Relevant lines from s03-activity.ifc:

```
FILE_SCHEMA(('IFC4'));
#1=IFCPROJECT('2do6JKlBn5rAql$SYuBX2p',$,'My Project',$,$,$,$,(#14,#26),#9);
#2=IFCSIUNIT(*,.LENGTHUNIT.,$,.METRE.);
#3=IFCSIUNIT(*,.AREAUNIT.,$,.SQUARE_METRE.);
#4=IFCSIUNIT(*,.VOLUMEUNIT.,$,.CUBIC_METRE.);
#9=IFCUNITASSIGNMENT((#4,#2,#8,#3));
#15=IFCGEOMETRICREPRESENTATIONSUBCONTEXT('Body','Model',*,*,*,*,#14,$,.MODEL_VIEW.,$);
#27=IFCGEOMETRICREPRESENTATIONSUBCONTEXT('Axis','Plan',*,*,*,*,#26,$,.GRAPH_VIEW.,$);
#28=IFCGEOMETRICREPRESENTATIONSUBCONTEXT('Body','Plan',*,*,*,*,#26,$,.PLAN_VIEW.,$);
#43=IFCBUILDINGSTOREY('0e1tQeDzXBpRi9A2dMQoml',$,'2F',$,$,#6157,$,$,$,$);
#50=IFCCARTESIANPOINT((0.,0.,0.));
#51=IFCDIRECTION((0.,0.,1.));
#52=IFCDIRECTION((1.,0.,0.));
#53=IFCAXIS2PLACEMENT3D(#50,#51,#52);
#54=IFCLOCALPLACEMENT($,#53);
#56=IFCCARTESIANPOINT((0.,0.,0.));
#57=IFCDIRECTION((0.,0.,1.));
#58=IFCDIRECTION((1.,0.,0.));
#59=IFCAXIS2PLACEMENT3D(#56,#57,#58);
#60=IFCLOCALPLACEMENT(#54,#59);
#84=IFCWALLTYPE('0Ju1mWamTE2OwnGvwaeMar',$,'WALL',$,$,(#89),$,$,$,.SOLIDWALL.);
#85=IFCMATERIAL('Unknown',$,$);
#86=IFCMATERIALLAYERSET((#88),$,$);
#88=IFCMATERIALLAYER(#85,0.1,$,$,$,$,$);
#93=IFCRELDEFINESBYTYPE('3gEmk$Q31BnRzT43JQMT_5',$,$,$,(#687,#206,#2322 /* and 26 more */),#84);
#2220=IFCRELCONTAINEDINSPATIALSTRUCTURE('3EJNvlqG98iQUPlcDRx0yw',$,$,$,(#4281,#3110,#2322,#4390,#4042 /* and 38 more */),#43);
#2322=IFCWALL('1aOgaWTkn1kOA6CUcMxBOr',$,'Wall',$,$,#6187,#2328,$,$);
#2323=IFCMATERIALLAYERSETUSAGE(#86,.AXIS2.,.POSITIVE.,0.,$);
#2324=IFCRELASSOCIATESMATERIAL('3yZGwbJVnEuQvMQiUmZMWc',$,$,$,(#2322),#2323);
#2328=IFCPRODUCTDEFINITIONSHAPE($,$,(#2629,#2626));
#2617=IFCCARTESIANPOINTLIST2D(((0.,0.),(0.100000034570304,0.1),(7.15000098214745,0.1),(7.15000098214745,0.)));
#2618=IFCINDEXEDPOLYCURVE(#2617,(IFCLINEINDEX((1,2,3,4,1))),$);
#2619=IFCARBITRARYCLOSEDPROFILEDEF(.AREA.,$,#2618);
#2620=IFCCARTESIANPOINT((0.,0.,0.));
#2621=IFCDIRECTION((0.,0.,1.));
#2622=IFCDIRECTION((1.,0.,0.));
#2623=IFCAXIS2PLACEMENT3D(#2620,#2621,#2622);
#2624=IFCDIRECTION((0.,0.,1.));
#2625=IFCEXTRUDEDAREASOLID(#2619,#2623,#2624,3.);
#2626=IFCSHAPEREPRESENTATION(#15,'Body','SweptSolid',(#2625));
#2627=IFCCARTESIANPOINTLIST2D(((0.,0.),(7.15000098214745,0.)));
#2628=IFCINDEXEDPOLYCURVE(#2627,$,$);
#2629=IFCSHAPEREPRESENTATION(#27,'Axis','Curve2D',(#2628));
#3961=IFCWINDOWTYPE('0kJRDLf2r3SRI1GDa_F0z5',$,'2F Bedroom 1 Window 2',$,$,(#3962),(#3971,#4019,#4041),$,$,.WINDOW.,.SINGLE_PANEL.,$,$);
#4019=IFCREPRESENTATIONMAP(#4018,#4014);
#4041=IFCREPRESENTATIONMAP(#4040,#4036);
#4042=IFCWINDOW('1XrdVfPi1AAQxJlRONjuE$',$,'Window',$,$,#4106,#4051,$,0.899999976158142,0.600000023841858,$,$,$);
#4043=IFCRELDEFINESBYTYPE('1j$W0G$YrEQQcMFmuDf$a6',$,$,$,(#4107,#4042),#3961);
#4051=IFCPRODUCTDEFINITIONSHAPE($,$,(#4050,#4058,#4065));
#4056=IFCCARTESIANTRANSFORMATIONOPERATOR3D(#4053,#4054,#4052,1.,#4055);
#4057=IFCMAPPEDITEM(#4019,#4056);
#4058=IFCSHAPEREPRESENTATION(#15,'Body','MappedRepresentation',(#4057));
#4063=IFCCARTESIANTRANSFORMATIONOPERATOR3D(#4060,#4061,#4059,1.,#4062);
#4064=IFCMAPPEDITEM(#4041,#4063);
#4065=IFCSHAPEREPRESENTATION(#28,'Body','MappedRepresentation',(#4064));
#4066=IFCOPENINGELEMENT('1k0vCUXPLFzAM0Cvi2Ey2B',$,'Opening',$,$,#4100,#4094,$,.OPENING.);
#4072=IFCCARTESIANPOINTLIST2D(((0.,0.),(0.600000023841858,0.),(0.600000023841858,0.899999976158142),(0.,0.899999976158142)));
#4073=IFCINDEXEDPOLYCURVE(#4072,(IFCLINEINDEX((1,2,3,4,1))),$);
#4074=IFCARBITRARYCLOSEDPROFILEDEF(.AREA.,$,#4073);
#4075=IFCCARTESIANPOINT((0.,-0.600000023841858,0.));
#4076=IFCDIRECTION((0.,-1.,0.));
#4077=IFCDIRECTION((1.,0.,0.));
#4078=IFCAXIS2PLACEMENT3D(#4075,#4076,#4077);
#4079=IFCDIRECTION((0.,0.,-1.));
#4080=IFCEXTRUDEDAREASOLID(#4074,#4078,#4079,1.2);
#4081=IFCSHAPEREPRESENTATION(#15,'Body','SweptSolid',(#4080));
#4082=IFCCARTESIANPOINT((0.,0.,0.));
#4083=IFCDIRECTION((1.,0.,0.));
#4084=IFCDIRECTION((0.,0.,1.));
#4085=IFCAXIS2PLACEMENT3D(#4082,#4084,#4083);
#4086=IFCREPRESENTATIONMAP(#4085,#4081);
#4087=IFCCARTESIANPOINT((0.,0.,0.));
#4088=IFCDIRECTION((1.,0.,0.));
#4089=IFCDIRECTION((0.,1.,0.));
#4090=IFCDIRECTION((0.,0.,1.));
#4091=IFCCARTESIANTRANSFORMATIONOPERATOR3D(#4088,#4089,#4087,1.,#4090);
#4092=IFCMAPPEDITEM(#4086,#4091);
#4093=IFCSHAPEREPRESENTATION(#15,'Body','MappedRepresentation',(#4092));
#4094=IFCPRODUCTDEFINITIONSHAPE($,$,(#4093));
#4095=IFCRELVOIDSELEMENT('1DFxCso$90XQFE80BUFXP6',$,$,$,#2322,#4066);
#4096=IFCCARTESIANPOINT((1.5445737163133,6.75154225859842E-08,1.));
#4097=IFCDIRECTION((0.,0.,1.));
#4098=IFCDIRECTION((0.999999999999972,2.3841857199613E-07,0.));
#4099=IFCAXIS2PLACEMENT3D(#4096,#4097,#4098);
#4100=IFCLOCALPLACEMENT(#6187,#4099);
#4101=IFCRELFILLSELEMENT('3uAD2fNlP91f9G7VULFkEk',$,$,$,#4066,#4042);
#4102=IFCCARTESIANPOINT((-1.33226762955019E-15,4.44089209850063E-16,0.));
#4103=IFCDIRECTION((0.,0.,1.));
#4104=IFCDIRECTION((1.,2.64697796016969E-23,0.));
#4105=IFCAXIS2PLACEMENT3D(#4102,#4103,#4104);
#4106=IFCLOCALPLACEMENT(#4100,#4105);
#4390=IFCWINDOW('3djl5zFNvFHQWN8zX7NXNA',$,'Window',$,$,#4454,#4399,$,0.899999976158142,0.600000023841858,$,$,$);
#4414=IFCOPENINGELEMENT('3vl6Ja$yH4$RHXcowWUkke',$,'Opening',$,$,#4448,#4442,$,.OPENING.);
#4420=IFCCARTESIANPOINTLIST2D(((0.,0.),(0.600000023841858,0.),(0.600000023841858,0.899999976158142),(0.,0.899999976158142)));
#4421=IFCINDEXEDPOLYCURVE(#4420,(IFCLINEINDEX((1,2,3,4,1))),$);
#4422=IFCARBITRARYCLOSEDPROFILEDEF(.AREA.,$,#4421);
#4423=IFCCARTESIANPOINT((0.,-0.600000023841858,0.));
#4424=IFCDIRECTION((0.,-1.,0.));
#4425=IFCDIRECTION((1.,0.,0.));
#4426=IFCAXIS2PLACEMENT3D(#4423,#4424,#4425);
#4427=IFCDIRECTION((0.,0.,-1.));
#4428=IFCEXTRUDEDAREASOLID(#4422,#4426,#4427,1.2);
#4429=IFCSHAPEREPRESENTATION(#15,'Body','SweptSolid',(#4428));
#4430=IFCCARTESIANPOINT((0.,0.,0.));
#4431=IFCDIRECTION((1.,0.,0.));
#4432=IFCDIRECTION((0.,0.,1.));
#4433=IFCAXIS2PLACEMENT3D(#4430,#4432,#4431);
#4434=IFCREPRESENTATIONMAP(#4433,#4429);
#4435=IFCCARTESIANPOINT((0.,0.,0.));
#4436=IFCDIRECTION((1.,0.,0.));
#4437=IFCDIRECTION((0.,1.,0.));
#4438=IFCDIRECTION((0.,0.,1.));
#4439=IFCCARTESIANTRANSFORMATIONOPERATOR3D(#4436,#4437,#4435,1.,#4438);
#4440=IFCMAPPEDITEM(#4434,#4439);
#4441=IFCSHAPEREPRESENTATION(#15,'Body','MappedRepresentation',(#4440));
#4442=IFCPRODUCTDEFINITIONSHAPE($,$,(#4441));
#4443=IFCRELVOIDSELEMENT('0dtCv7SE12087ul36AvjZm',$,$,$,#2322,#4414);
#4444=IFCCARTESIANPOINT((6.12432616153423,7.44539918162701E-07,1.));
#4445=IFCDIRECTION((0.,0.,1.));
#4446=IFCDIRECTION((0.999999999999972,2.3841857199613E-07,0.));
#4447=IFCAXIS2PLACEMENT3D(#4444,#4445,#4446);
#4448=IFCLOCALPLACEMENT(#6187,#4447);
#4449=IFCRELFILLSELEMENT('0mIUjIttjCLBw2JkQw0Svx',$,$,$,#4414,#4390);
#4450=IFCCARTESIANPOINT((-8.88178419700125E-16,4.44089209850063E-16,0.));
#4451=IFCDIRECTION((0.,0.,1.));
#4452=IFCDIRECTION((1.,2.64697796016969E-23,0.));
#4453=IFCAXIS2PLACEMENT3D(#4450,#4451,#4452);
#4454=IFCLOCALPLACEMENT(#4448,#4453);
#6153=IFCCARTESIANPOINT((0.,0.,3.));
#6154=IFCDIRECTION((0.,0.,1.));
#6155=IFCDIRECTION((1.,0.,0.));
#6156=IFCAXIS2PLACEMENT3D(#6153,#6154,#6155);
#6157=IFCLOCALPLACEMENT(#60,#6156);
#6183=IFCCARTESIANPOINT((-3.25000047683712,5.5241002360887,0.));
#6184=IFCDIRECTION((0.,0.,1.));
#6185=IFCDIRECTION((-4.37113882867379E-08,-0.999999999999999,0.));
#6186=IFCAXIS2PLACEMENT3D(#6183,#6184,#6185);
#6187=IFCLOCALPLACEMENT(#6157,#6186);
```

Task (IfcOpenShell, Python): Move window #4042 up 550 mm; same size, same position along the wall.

```python
import numpy as np
import ifcopenshell
import ifcopenshell.api.geometry
import ifcopenshell.util.placement
import ifcopenshell.util.unit

model = ifcopenshell.open("s03-activity.ifc")
unit_scale = ifcopenshell.util.unit.calculate_unit_scale(model)

window = model.by_guid("1XrdVfPi1AAQxJlRONjuE$")
opening = window.FillsVoids[0].RelatingOpeningElement
dz = 0.55 / unit_scale

shift = np.array([0.0, 0.0, dz])
# The window is placed relative to its opening, so it follows when the opening moves.
matrix = ifcopenshell.util.placement.get_local_placement(opening.ObjectPlacement)
matrix[:3, 3] += shift
ifcopenshell.api.geometry.edit_object_placement(
    model, product=opening, matrix=matrix, is_si=False, should_transform_children=True
)

print(f"moved by {dz * unit_scale:+.3f} m")

model.write("s03-activity_v2.ifc")
```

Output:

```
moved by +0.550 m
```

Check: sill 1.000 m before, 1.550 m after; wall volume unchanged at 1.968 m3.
